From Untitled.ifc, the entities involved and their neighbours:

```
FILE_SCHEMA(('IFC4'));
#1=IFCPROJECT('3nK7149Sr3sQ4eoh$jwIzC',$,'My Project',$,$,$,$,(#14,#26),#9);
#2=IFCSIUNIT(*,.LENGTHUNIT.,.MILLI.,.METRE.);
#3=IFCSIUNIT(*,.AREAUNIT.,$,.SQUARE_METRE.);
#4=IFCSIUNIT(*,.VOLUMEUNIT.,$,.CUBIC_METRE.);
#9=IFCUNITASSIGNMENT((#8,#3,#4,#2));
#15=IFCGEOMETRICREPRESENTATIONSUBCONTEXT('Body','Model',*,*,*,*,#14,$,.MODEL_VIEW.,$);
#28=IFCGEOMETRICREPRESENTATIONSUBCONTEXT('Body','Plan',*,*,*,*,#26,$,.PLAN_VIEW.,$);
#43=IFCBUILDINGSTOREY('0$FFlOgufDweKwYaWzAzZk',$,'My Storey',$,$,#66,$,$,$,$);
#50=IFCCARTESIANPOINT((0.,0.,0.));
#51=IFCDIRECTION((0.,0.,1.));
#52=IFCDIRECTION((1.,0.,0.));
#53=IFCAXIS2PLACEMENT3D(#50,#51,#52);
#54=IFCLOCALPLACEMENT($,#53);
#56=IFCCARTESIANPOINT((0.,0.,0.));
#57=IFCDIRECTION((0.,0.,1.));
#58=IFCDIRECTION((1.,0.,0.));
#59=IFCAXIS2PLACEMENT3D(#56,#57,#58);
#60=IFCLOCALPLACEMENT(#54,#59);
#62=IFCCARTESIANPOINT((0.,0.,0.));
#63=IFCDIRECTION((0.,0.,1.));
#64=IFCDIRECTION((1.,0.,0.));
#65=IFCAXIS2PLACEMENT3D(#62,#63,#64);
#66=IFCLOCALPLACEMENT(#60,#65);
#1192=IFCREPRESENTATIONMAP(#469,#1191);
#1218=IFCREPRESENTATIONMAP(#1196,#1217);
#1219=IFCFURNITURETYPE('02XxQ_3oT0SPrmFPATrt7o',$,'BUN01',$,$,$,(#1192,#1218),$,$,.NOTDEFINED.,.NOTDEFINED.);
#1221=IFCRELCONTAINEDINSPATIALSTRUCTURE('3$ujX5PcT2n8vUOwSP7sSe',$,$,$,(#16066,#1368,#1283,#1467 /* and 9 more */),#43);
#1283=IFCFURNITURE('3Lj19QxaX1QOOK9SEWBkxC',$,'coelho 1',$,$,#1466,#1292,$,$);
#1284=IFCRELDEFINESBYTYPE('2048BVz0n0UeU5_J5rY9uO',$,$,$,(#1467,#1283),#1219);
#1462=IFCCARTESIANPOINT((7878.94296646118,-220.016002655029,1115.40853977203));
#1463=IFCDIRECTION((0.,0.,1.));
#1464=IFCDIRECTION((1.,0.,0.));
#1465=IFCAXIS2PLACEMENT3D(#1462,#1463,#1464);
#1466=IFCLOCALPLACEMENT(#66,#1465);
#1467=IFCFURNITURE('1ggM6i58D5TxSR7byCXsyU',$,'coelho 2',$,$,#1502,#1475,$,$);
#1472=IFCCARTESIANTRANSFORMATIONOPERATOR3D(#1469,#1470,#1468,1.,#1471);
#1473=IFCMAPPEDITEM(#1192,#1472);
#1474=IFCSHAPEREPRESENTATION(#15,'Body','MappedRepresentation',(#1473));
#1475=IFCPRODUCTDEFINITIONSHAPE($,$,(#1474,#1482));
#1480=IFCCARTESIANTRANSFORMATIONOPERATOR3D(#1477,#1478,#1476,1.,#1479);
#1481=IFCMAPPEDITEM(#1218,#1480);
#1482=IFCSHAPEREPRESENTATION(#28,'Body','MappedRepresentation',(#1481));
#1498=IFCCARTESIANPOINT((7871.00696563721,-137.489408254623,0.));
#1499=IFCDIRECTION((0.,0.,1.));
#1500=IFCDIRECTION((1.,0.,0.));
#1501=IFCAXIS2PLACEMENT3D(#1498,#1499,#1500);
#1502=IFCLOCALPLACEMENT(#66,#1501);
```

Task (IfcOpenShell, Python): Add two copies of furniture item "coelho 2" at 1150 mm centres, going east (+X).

```python
import numpy as np
import ifcopenshell
import ifcopenshell.api.geometry
import ifcopenshell.api.root
import ifcopenshell.util.element
import ifcopenshell.util.placement
import ifcopenshell.util.unit

model = ifcopenshell.open("Untitled.ifc")
unit_scale = ifcopenshell.util.unit.calculate_unit_scale(model)

source = model.by_guid("1ggM6i58D5TxSR7byCXsyU")
base = ifcopenshell.util.placement.get_local_placement(source.ObjectPlacement)
step = np.array([1.0, 0.0, 0.0]) * 1.15 / unit_scale

for i in range(1, 3):
    copy = ifcopenshell.api.root.copy_class(model, product=source)
    copy.Representation = ifcopenshell.util.element.copy_deep(
        model, source.Representation, exclude=["IfcGeometricRepresentationContext", "IfcRepresentationMap"]
    )
    matrix = base.copy()
    matrix[:3, 3] += i * step
    print("added at", matrix[:3, 3].round(3) + 0.0)
    ifcopenshell.api.geometry.edit_object_placement(model, product=copy, matrix=matrix, is_si=False)

model.write("Untitled-out.ifc")
```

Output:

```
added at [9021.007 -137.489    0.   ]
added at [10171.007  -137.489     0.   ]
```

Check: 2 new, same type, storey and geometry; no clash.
